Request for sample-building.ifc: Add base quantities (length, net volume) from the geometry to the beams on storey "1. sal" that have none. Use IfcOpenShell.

First a look at what the model holds.

```python
import ifcopenshell
import ifcopenshell.util.element
import ifcopenshell.util.unit

model = ifcopenshell.open("sample-building.ifc")
print(model.schema)
for unit_type in ("LENGTHUNIT", "AREAUNIT", "VOLUMEUNIT"):
    print(unit_type, ifcopenshell.util.unit.calculate_unit_scale(model, unit_type))
storey = next(s for s in model.by_type("IfcBuildingStorey") if s.Name == "1. sal")
beams = [e for e in ifcopenshell.util.element.get_decomposition(storey) if e.is_a("IfcBeam")]
for e in sorted(beams, key=lambda e: e.id()):
    print(e.id(), e.is_a(), e.Name, list(ifcopenshell.util.element.get_psets(e, qtos_only=True)), sep=" | ")
```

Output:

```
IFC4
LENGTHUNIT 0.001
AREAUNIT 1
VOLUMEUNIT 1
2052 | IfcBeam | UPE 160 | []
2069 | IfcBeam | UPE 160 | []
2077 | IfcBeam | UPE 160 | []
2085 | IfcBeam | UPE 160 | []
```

```python
import ifcopenshell
import ifcopenshell.api.pset
import ifcopenshell.geom
import ifcopenshell.util.element
import ifcopenshell.util.shape
import ifcopenshell.util.unit

model = ifcopenshell.open("sample-building.ifc")
unit_scale = ifcopenshell.util.unit.calculate_unit_scale(model)
volume_scale = ifcopenshell.util.unit.calculate_unit_scale(model, "VOLUMEUNIT")
settings = ifcopenshell.geom.settings()

storey = next(s for s in model.by_type("IfcBuildingStorey") if s.Name == "1. sal")
beams = [e for e in ifcopenshell.util.element.get_decomposition(storey) if e.is_a("IfcBeam")]

for e in sorted(beams, key=lambda e: e.id()):
    if ifcopenshell.util.element.get_psets(e, qtos_only=True, should_inherit=False):
        continue
    # Geometry comes back in metres, in the element's own axes.
    shape = ifcopenshell.geom.create_shape(settings, e)
    values = {
        "Length": ifcopenshell.util.shape.get_max_xyz(shape.geometry) / unit_scale,
        "NetVolume": ifcopenshell.util.shape.get_volume(shape.geometry) / volume_scale,
    }
    qto = ifcopenshell.api.pset.add_qto(model, product=e, name="Qto_BeamBaseQuantities")
    ifcopenshell.api.pset.edit_qto(model, qto=qto, properties=values)
    print(e.id(), {k: round(v, 3) for k, v in values.items()})

model.write("sample-building_v2.ifc")
```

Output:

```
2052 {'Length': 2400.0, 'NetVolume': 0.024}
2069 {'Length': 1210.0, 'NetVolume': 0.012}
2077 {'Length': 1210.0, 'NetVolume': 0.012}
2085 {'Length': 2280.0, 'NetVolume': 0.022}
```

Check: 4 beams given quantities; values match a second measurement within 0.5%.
